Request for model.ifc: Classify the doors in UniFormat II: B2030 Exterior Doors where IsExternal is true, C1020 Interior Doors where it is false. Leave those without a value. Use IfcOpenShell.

First a look at what the model holds.

```python
import ifcopenshell
import ifcopenshell.util.element

model = ifcopenshell.open("model.ifc")
print(model.schema)
print("classifications:", [c.Name for c in model.by_type("IfcClassification")])
values = [ifcopenshell.util.element.get_pset(e, "Pset_DoorCommon", "IsExternal") for e in model.by_type("IfcDoor")]
for value in (True, False, None):
    print("IsExternal", value, values.count(value))
```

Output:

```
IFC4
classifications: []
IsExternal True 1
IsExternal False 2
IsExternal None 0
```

```python
import ifcopenshell
import ifcopenshell.api.classification
import ifcopenshell.util.element

model = ifcopenshell.open("model.ifc")

system = ifcopenshell.api.classification.add_classification(model, classification="UniFormat II")

doors = model.by_type("IfcDoor")
external = {e: ifcopenshell.util.element.get_pset(e, "Pset_DoorCommon", "IsExternal") for e in doors}
for flag, code, name in ((True, "B2030", "Exterior Doors"), (False, "C1020", "Interior Doors")):
    products = [e for e in doors if external[e] is flag]
    ifcopenshell.api.classification.add_reference(
        model, products=products, classification=system, identification=code, name=name
    )
    print(code, len(products))

model.write("model-out.ifc")
```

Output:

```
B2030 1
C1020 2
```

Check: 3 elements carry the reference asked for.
